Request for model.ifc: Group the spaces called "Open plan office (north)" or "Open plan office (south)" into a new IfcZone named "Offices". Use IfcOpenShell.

First a look at what the model holds.

```python
import ifcopenshell

model = ifcopenshell.open("model.ifc")
print(model.schema)
seen = {}
for space in model.by_type("IfcSpace"):
    seen[space.LongName] = seen.get(space.LongName, 0) + 1
for name, count in sorted(seen.items(), key=str):
    print(count, "x", name)
print("zones:", [z.Name for z in model.by_type("IfcZone")][:20])
```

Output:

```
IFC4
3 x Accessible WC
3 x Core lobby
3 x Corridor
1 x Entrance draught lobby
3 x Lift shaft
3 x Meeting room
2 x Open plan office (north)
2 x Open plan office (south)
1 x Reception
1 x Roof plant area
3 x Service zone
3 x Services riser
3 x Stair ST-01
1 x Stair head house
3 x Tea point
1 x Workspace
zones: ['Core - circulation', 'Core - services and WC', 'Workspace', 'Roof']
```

```python
import ifcopenshell
import ifcopenshell.api.group
import ifcopenshell.api.root

model = ifcopenshell.open("model.ifc")

names = {"Open plan office (north)", "Open plan office (south)"}
spaces = [s for s in model.by_type("IfcSpace") if s.LongName in names]

zone = ifcopenshell.api.root.create_entity(model, ifc_class="IfcZone", name="Offices")
ifcopenshell.api.group.assign_group(model, products=spaces, group=zone)
print(len(spaces), "spaces in", zone.Name)

model.write("model_edited.ifc")
```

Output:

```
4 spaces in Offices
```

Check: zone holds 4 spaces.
